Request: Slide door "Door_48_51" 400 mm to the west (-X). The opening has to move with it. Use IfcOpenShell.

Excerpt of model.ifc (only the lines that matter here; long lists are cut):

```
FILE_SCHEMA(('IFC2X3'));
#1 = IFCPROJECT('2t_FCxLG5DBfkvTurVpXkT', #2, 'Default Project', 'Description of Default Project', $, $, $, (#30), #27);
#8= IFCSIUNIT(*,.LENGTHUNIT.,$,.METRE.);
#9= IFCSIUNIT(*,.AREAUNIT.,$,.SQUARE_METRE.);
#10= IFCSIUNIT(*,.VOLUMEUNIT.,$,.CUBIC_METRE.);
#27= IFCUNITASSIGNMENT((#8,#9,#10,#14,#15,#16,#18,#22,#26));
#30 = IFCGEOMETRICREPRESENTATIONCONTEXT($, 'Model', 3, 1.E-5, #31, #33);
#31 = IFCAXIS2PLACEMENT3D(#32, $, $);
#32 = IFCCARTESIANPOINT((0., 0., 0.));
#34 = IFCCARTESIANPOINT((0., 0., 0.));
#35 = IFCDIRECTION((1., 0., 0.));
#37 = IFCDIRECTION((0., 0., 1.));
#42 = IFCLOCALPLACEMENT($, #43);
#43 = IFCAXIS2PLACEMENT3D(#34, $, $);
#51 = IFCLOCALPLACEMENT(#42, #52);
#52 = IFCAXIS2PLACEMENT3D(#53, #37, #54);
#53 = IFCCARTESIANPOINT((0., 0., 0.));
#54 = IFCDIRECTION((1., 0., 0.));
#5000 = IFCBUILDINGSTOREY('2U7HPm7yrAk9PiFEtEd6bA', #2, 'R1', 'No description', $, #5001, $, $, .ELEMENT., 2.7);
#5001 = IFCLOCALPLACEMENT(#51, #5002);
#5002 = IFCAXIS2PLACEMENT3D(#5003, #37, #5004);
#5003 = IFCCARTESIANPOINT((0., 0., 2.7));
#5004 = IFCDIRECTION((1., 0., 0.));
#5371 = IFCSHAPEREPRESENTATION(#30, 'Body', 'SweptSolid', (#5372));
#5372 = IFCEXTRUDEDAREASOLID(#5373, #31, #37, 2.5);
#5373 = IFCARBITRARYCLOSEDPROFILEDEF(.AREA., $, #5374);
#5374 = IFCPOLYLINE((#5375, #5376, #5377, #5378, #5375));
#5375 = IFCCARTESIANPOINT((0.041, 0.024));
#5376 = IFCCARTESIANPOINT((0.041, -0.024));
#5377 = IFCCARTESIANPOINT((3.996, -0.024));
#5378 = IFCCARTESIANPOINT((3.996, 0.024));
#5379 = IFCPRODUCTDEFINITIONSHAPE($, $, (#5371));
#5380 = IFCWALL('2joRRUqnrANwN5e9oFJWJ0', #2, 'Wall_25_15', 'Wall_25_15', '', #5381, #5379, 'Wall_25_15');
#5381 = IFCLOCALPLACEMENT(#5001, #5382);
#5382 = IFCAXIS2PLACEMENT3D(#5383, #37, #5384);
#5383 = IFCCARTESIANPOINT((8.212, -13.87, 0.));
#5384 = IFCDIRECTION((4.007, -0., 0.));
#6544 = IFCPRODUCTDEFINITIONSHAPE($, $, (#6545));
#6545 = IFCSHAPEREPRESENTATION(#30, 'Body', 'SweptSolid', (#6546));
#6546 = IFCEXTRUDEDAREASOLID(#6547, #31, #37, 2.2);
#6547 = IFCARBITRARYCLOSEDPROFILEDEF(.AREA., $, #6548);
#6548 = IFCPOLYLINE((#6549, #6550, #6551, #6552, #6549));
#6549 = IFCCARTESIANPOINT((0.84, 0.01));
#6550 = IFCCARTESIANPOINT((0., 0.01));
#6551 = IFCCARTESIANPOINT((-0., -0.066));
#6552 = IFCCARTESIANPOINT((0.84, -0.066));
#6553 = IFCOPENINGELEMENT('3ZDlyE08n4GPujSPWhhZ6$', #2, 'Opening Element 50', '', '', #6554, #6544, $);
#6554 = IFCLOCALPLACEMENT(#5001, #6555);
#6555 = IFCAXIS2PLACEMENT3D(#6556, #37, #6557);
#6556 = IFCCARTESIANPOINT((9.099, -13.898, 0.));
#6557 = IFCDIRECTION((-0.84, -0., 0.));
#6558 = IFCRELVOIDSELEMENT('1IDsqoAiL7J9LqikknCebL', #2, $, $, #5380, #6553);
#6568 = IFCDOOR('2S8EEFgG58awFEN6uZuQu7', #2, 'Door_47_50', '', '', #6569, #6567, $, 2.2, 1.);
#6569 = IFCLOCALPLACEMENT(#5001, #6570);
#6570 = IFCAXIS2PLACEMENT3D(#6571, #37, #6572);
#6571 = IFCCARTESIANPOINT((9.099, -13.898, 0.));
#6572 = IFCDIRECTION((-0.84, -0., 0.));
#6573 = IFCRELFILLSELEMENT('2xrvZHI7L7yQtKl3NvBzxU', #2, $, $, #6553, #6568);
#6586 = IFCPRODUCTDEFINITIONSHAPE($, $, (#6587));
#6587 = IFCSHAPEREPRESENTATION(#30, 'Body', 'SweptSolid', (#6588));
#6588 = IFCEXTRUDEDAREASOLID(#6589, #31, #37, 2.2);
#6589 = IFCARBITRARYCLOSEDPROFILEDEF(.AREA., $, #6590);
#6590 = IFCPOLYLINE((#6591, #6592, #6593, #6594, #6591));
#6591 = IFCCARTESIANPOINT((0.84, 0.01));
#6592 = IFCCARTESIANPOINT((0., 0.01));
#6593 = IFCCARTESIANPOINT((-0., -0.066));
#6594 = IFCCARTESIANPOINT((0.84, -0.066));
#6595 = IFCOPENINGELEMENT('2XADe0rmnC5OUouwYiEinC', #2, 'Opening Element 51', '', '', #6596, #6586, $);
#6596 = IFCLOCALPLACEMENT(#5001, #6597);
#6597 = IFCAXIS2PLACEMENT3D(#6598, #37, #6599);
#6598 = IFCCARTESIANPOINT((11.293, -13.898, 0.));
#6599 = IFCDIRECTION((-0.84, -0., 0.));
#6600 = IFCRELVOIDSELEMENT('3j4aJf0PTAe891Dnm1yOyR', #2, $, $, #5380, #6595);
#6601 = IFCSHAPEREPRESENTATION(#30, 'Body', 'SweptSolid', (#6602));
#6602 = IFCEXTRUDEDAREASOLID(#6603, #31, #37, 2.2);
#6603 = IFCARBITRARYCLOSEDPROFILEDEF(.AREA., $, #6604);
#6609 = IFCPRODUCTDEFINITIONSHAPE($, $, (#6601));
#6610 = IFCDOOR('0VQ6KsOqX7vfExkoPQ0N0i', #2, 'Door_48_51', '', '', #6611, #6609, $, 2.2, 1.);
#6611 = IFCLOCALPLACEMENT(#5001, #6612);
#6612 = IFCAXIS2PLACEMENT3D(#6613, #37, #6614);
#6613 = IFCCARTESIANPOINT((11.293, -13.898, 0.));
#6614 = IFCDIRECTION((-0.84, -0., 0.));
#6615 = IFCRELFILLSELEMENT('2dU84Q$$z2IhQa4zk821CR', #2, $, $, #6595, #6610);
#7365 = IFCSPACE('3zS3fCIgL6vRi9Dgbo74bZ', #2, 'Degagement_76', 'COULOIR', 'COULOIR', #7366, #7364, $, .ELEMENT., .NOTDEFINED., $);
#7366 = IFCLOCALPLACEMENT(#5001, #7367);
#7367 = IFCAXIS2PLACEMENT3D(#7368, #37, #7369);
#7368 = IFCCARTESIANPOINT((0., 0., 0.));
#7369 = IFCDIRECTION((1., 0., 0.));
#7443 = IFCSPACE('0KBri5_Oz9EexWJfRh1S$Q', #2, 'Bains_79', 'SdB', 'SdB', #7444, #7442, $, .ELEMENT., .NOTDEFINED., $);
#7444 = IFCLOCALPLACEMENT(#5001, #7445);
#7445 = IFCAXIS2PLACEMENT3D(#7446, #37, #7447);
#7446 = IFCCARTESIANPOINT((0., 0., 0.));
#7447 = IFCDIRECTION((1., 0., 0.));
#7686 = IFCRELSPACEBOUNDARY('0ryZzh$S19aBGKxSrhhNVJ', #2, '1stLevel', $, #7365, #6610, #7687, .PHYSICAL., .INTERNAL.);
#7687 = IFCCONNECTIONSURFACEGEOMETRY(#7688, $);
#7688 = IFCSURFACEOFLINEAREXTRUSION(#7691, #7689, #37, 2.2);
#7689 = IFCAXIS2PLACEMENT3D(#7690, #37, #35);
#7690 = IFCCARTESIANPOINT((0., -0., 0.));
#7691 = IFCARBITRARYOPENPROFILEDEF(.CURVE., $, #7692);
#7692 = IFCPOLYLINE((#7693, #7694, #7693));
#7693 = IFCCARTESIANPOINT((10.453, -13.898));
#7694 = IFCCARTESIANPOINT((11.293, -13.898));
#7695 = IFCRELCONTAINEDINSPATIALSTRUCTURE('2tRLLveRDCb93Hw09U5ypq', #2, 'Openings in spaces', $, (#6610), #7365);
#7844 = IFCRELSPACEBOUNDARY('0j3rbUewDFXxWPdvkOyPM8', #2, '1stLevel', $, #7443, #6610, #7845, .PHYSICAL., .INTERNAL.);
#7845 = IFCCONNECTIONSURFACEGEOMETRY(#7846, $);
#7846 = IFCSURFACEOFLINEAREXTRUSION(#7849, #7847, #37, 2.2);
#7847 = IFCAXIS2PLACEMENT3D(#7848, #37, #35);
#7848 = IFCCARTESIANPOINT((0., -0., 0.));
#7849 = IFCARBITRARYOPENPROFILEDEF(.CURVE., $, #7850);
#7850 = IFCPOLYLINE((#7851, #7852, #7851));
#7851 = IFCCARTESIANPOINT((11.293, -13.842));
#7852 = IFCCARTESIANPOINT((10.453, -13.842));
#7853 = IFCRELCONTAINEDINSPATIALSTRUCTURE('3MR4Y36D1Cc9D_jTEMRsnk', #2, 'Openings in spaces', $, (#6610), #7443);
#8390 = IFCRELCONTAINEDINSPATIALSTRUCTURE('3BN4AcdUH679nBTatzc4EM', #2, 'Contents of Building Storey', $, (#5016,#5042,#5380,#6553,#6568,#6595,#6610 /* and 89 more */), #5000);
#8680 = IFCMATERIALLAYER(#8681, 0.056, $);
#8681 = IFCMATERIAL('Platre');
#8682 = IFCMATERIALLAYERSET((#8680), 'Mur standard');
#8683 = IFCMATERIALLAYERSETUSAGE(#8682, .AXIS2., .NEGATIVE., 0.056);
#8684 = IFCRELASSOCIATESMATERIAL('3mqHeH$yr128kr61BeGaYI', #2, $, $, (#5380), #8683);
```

```python
import numpy as np
import ifcopenshell
import ifcopenshell.api.geometry
import ifcopenshell.util.placement

model = ifcopenshell.open("model.ifc")

door = model.by_guid("0VQ6KsOqX7vfExkoPQ0N0i")
opening = door.FillsVoids[0].RelatingOpeningElement
wall = opening.VoidsElements[0].RelatingBuildingElement

wall_matrix = ifcopenshell.util.placement.get_local_placement(wall.ObjectPlacement)
shift = wall_matrix[:3, 0] * -0.4
before = ifcopenshell.util.placement.get_local_placement(door.ObjectPlacement)[:3, 3].copy()

# The door is not placed relative to its opening, so move both.
for product in (opening, door):
    matrix = ifcopenshell.util.placement.get_local_placement(product.ObjectPlacement)
    matrix[:3, 3] += shift
    ifcopenshell.api.geometry.edit_object_placement(model, product=product, matrix=matrix, is_si=False)

# Space boundary surfaces are stored in each space's coordinates; move them too.
for rel in door.ProvidesBoundaries:
    if not rel.ConnectionGeometry:
        continue
    surface = rel.ConnectionGeometry.SurfaceOnRelatingElement
    space_matrix = ifcopenshell.util.placement.get_local_placement(rel.RelatingSpace.ObjectPlacement)
    point = np.array(surface.Position.Location.Coordinates) + space_matrix[:3, :3].T @ shift
    surface.Position = model.createIfcAxis2Placement3D(
        model.createIfcCartesianPoint(point.tolist()), surface.Position.Axis, surface.Position.RefDirection
    )

after = ifcopenshell.util.placement.get_local_placement(door.ObjectPlacement)[:3, 3]
print("door moved by", (after - before).round(3) + 0.0)

model.write("model-out.ifc")
```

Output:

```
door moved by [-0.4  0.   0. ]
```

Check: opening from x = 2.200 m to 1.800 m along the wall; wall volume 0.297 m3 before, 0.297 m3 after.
